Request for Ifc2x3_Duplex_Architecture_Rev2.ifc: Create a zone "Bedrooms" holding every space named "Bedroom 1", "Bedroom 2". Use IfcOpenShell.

First a look at what the model holds.

```python
import ifcopenshell

model = ifcopenshell.open("Ifc2x3_Duplex_Architecture_Rev2.ifc")
print(model.schema)
seen = {}
for space in model.by_type("IfcSpace"):
    seen[space.LongName] = seen.get(space.LongName, 0) + 1
for name, count in sorted(seen.items(), key=str):
    print(count, "x", name)
print("zones:", [z.Name for z in model.by_type("IfcZone")][:20])
```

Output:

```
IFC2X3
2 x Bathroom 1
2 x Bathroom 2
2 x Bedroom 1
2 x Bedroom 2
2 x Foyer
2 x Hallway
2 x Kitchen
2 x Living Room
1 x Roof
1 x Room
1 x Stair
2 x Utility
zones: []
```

```python
import ifcopenshell
import ifcopenshell.api.group
import ifcopenshell.api.root

model = ifcopenshell.open("Ifc2x3_Duplex_Architecture_Rev2.ifc")

names = {"Bedroom 1", "Bedroom 2"}
spaces = [s for s in model.by_type("IfcSpace") if s.LongName in names]

zone = ifcopenshell.api.root.create_entity(model, ifc_class="IfcZone", name="Bedrooms")
ifcopenshell.api.group.assign_group(model, products=spaces, group=zone)
print(len(spaces), "spaces in", zone.Name)

model.write("Ifc2x3_Duplex_Architecture_Rev2_rev.ifc")
```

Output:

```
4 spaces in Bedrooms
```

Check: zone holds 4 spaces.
